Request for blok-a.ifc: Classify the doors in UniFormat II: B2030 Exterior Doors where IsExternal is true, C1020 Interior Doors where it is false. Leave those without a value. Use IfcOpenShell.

First a look at what the model holds.

```python
import ifcopenshell
import ifcopenshell.util.element

model = ifcopenshell.open("blok-a.ifc")
print(model.schema)
print("classifications:", [c.Name for c in model.by_type("IfcClassification")])
values = [ifcopenshell.util.element.get_pset(e, "Pset_DoorCommon", "IsExternal") for e in model.by_type("IfcDoor")]
for value in (True, False, None):
    print("IsExternal", value, values.count(value))
```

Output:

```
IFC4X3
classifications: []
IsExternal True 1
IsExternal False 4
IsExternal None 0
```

```python
import ifcopenshell
import ifcopenshell.api.classification
import ifcopenshell.util.element

model = ifcopenshell.open("blok-a.ifc")

system = ifcopenshell.api.classification.add_classification(model, classification="UniFormat II")

doors = model.by_type("IfcDoor")
external = {e: ifcopenshell.util.element.get_pset(e, "Pset_DoorCommon", "IsExternal") for e in doors}
for flag, code, name in ((True, "B2030", "Exterior Doors"), (False, "C1020", "Interior Doors")):
    products = [e for e in doors if external[e] is flag]
    ifcopenshell.api.classification.add_reference(
        model, products=products, classification=system, identification=code, name=name
    )
    print(code, len(products))

model.write("blok-a_edited.ifc")
```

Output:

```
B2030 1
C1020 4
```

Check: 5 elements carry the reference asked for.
